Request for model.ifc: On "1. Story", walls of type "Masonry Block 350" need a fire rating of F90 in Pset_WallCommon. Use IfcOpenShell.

First a look at what the model holds.

```python
import ifcopenshell
import ifcopenshell.util.element

model = ifcopenshell.open("model.ifc")
print(model.schema)
storey = next(s for s in model.by_type("IfcBuildingStorey") if s.Name == "1. Story")
walls = [e for e in ifcopenshell.util.element.get_decomposition(storey) if e.is_a("IfcWall")]
seen = {}
for e in walls:
    element_type = ifcopenshell.util.element.get_type(e)
    key = (element_type.Name if element_type != e and element_type else None, ifcopenshell.util.element.get_pset(e, "Pset_WallCommon", "FireRating"))
    seen[key] = seen.get(key, 0) + 1
for (name, value), count in sorted(seen.items(), key=str):
    print(count, "x", name, "|", value)
```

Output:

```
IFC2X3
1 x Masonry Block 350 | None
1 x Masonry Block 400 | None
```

```python
import ifcopenshell
import ifcopenshell.api.pset
import ifcopenshell.util.element

model = ifcopenshell.open("model.ifc")

storey = next(s for s in model.by_type("IfcBuildingStorey") if s.Name == "1. Story")
walls = [e for e in ifcopenshell.util.element.get_decomposition(storey) if e.is_a("IfcWall")]

count = 0
for e in walls:
    element_type = ifcopenshell.util.element.get_type(e)
    if element_type in (None, e) or element_type.Name != "Masonry Block 350":
        continue
    # add_pset returns the element's existing set when there is one.
    pset = ifcopenshell.api.pset.add_pset(model, product=e, name="Pset_WallCommon")
    ifcopenshell.api.pset.edit_pset(model, pset=pset, properties={"FireRating": "F90"})
    count += 1

print(count, "walls updated")

model.write("model_edited.ifc")
```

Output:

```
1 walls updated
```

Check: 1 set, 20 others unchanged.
